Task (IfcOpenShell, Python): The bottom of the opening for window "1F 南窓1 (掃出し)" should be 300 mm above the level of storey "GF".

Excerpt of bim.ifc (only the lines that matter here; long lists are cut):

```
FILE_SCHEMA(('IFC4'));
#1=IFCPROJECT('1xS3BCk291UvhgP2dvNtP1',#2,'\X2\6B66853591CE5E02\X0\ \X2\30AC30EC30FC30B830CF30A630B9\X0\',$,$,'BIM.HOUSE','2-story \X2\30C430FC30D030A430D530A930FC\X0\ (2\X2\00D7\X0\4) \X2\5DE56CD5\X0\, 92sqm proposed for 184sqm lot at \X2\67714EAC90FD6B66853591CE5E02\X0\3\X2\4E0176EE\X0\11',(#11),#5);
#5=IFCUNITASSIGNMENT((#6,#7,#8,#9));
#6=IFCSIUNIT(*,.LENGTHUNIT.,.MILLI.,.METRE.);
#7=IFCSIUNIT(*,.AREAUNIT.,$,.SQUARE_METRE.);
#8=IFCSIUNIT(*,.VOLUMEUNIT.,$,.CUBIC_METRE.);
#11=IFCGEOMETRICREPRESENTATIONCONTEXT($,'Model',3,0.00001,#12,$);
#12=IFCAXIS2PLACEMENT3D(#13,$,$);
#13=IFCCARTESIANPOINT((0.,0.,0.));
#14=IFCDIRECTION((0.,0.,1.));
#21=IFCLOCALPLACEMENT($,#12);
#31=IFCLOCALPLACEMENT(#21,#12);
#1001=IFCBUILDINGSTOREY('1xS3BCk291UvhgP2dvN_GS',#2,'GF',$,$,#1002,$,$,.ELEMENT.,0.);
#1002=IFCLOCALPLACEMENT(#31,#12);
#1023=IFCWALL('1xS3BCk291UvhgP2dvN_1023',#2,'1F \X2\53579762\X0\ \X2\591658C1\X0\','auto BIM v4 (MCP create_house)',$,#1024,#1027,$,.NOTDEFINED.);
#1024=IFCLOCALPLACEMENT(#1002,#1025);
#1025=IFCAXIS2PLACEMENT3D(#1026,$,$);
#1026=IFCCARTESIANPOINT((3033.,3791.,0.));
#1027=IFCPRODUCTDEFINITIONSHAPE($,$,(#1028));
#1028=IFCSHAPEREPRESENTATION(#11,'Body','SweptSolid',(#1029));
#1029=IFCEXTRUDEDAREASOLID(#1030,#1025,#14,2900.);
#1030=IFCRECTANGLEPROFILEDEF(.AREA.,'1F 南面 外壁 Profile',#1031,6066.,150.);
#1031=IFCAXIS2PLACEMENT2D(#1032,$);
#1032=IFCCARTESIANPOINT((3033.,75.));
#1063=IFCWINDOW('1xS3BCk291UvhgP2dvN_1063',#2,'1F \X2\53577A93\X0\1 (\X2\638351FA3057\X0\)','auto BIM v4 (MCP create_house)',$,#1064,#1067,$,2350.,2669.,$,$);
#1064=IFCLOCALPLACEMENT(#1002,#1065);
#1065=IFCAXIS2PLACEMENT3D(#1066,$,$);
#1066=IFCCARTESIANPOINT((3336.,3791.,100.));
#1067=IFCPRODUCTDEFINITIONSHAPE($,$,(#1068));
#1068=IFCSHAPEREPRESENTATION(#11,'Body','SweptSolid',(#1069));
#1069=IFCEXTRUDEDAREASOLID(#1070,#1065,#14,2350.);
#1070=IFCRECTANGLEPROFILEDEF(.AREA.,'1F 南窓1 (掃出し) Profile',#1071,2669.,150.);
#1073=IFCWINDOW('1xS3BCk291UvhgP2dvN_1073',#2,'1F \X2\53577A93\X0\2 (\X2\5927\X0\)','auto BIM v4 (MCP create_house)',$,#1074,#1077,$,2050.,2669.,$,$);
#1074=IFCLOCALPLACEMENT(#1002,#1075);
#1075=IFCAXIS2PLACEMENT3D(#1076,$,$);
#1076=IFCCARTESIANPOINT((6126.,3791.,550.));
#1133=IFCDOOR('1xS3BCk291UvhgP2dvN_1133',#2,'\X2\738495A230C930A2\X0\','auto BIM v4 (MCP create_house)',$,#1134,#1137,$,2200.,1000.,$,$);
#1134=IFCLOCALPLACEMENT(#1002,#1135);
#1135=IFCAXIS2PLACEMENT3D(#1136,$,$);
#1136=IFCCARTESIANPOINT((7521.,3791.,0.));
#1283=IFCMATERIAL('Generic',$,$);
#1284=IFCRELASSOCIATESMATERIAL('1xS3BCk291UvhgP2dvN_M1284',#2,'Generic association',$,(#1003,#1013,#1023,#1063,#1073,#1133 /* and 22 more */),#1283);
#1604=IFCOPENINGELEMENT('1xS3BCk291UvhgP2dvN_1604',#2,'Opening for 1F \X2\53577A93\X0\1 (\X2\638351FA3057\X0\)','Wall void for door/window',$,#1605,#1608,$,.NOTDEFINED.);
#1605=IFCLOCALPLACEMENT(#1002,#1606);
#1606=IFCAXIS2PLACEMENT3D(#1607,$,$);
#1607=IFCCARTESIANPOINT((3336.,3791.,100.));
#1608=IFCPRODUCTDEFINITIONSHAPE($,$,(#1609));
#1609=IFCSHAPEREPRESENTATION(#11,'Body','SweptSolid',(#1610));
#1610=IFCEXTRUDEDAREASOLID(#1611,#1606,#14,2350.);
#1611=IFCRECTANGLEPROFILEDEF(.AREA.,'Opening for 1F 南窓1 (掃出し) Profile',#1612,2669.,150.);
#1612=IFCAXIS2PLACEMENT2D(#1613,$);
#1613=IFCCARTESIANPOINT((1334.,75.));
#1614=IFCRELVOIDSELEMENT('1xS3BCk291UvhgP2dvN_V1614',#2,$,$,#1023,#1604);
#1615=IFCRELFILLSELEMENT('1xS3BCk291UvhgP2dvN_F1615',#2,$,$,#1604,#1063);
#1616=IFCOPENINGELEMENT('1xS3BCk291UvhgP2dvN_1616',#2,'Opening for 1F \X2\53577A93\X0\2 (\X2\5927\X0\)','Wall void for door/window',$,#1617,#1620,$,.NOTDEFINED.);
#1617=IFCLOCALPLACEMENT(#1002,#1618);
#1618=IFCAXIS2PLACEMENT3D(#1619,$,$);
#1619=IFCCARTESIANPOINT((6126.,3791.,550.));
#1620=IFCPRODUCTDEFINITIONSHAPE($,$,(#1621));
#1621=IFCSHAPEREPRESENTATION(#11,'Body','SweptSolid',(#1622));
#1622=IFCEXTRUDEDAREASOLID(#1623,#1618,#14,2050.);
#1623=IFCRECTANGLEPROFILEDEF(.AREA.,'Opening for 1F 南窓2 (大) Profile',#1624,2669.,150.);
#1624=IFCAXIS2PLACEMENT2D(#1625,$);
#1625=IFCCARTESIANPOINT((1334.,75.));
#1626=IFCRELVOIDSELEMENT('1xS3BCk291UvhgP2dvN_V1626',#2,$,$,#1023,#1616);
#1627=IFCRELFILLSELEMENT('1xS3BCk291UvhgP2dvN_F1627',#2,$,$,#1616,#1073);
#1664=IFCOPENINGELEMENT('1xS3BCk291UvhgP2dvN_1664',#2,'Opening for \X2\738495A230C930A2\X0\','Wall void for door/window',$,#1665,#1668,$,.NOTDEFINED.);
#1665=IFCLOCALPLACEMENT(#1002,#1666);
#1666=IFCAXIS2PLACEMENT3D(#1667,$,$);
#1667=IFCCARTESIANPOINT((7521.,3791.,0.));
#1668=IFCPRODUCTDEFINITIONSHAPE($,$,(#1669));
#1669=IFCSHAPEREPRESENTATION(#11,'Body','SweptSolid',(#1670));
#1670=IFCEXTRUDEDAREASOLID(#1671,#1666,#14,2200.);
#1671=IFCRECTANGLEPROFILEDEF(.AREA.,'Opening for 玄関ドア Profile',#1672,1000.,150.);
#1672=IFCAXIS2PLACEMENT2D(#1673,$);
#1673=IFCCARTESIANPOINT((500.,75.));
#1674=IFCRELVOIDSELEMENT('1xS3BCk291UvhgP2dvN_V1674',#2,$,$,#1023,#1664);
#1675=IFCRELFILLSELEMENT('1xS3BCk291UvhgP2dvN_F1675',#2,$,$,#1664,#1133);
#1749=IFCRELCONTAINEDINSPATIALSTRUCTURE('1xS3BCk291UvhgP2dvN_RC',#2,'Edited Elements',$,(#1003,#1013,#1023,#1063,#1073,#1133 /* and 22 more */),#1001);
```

```python
import numpy as np
import ifcopenshell
import ifcopenshell.api.geometry
import ifcopenshell.geom
import ifcopenshell.util.element
import ifcopenshell.util.placement
import ifcopenshell.util.shape
import ifcopenshell.util.unit

model = ifcopenshell.open("bim.ifc")
unit_scale = ifcopenshell.util.unit.calculate_unit_scale(model)

window = model.by_guid("1xS3BCk291UvhgP2dvN_1063")
opening = window.FillsVoids[0].RelatingOpeningElement
storey = ifcopenshell.util.element.get_container(window, ifc_class="IfcBuildingStorey")
level = ifcopenshell.util.placement.get_local_placement(storey.ObjectPlacement)[2, 3]

# The opening's origin need not be at the sill, so measure its lowest point.
shape = ifcopenshell.geom.create_shape(ifcopenshell.geom.settings(), opening)
bottom = ifcopenshell.util.shape.get_shape_bottom_elevation(shape, shape.geometry) / unit_scale
dz = level + 300.0 - bottom

shift = np.array([0.0, 0.0, dz])
# The window is not placed relative to its opening, so move both.
for product in (opening, window):
    matrix = ifcopenshell.util.placement.get_local_placement(product.ObjectPlacement)
    matrix[:3, 3] += shift
    ifcopenshell.api.geometry.edit_object_placement(model, product=product, matrix=matrix, is_si=False)

print(f"moved by {dz * unit_scale:+.3f} m")

model.write("bim_edited.ifc")
```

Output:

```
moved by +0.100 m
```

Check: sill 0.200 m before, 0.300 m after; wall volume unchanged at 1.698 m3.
